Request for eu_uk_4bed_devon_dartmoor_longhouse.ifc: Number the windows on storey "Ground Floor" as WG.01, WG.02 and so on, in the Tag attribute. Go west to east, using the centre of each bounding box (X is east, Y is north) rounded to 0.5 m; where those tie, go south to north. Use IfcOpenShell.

First a look at what the model holds.

```python
import ifcopenshell
import ifcopenshell.util.element
import ifcopenshell.util.placement

model = ifcopenshell.open("eu_uk_4bed_devon_dartmoor_longhouse.ifc")
print(model.schema)
storey = next(s for s in model.by_type("IfcBuildingStorey") if s.Name == "Ground Floor")
windows = [e for e in ifcopenshell.util.element.get_decomposition(storey) if e.is_a("IfcWindow")]
for e in sorted(windows, key=lambda e: e.id()):
    origin = ifcopenshell.util.placement.get_local_placement(e.ObjectPlacement)[:3, 3]
    print(e.id(), e.Tag, e.Name, origin.round(2) + 0.0, sep=" | ")
```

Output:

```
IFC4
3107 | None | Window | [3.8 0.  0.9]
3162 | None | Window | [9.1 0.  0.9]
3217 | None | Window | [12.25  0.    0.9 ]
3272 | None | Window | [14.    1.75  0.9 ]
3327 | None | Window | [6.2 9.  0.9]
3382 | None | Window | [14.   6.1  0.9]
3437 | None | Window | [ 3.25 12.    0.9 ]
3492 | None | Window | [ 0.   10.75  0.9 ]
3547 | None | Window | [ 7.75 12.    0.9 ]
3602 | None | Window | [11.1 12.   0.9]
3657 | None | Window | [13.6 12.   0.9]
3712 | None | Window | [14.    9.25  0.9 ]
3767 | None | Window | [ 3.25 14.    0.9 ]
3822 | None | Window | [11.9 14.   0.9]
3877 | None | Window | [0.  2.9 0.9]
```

```python
import ifcopenshell
import ifcopenshell.geom
import ifcopenshell.util.element
import ifcopenshell.util.shape

model = ifcopenshell.open("eu_uk_4bed_devon_dartmoor_longhouse.ifc")
settings = ifcopenshell.geom.settings()
settings.set("use-world-coords", True)


def centre(element):
    shape = ifcopenshell.geom.create_shape(settings, element)
    return ifcopenshell.util.shape.get_bbox_centroid(shape.geometry)


storey = next(s for s in model.by_type("IfcBuildingStorey") if s.Name == "Ground Floor")
windows = [e for e in ifcopenshell.util.element.get_decomposition(storey) if e.is_a("IfcWindow")]

# Insertion points can sit at a corner or the storey origin, so sort by the geometry (in metres).
centres = {e: centre(e) for e in windows}
windows.sort(key=lambda e: (round(centres[e][0] / 0.5), centres[e][1]))

for i, e in enumerate(windows, start=1):
    number = f"WG.{i:02d}"
    e.Tag = number
    print(e.id(), number)

model.write("eu_uk_4bed_devon_dartmoor_longhouse-out.ifc")
```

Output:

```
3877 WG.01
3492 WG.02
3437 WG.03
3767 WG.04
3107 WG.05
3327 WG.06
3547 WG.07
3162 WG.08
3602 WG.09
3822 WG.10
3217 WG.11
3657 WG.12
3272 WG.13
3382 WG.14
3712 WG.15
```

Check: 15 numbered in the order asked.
